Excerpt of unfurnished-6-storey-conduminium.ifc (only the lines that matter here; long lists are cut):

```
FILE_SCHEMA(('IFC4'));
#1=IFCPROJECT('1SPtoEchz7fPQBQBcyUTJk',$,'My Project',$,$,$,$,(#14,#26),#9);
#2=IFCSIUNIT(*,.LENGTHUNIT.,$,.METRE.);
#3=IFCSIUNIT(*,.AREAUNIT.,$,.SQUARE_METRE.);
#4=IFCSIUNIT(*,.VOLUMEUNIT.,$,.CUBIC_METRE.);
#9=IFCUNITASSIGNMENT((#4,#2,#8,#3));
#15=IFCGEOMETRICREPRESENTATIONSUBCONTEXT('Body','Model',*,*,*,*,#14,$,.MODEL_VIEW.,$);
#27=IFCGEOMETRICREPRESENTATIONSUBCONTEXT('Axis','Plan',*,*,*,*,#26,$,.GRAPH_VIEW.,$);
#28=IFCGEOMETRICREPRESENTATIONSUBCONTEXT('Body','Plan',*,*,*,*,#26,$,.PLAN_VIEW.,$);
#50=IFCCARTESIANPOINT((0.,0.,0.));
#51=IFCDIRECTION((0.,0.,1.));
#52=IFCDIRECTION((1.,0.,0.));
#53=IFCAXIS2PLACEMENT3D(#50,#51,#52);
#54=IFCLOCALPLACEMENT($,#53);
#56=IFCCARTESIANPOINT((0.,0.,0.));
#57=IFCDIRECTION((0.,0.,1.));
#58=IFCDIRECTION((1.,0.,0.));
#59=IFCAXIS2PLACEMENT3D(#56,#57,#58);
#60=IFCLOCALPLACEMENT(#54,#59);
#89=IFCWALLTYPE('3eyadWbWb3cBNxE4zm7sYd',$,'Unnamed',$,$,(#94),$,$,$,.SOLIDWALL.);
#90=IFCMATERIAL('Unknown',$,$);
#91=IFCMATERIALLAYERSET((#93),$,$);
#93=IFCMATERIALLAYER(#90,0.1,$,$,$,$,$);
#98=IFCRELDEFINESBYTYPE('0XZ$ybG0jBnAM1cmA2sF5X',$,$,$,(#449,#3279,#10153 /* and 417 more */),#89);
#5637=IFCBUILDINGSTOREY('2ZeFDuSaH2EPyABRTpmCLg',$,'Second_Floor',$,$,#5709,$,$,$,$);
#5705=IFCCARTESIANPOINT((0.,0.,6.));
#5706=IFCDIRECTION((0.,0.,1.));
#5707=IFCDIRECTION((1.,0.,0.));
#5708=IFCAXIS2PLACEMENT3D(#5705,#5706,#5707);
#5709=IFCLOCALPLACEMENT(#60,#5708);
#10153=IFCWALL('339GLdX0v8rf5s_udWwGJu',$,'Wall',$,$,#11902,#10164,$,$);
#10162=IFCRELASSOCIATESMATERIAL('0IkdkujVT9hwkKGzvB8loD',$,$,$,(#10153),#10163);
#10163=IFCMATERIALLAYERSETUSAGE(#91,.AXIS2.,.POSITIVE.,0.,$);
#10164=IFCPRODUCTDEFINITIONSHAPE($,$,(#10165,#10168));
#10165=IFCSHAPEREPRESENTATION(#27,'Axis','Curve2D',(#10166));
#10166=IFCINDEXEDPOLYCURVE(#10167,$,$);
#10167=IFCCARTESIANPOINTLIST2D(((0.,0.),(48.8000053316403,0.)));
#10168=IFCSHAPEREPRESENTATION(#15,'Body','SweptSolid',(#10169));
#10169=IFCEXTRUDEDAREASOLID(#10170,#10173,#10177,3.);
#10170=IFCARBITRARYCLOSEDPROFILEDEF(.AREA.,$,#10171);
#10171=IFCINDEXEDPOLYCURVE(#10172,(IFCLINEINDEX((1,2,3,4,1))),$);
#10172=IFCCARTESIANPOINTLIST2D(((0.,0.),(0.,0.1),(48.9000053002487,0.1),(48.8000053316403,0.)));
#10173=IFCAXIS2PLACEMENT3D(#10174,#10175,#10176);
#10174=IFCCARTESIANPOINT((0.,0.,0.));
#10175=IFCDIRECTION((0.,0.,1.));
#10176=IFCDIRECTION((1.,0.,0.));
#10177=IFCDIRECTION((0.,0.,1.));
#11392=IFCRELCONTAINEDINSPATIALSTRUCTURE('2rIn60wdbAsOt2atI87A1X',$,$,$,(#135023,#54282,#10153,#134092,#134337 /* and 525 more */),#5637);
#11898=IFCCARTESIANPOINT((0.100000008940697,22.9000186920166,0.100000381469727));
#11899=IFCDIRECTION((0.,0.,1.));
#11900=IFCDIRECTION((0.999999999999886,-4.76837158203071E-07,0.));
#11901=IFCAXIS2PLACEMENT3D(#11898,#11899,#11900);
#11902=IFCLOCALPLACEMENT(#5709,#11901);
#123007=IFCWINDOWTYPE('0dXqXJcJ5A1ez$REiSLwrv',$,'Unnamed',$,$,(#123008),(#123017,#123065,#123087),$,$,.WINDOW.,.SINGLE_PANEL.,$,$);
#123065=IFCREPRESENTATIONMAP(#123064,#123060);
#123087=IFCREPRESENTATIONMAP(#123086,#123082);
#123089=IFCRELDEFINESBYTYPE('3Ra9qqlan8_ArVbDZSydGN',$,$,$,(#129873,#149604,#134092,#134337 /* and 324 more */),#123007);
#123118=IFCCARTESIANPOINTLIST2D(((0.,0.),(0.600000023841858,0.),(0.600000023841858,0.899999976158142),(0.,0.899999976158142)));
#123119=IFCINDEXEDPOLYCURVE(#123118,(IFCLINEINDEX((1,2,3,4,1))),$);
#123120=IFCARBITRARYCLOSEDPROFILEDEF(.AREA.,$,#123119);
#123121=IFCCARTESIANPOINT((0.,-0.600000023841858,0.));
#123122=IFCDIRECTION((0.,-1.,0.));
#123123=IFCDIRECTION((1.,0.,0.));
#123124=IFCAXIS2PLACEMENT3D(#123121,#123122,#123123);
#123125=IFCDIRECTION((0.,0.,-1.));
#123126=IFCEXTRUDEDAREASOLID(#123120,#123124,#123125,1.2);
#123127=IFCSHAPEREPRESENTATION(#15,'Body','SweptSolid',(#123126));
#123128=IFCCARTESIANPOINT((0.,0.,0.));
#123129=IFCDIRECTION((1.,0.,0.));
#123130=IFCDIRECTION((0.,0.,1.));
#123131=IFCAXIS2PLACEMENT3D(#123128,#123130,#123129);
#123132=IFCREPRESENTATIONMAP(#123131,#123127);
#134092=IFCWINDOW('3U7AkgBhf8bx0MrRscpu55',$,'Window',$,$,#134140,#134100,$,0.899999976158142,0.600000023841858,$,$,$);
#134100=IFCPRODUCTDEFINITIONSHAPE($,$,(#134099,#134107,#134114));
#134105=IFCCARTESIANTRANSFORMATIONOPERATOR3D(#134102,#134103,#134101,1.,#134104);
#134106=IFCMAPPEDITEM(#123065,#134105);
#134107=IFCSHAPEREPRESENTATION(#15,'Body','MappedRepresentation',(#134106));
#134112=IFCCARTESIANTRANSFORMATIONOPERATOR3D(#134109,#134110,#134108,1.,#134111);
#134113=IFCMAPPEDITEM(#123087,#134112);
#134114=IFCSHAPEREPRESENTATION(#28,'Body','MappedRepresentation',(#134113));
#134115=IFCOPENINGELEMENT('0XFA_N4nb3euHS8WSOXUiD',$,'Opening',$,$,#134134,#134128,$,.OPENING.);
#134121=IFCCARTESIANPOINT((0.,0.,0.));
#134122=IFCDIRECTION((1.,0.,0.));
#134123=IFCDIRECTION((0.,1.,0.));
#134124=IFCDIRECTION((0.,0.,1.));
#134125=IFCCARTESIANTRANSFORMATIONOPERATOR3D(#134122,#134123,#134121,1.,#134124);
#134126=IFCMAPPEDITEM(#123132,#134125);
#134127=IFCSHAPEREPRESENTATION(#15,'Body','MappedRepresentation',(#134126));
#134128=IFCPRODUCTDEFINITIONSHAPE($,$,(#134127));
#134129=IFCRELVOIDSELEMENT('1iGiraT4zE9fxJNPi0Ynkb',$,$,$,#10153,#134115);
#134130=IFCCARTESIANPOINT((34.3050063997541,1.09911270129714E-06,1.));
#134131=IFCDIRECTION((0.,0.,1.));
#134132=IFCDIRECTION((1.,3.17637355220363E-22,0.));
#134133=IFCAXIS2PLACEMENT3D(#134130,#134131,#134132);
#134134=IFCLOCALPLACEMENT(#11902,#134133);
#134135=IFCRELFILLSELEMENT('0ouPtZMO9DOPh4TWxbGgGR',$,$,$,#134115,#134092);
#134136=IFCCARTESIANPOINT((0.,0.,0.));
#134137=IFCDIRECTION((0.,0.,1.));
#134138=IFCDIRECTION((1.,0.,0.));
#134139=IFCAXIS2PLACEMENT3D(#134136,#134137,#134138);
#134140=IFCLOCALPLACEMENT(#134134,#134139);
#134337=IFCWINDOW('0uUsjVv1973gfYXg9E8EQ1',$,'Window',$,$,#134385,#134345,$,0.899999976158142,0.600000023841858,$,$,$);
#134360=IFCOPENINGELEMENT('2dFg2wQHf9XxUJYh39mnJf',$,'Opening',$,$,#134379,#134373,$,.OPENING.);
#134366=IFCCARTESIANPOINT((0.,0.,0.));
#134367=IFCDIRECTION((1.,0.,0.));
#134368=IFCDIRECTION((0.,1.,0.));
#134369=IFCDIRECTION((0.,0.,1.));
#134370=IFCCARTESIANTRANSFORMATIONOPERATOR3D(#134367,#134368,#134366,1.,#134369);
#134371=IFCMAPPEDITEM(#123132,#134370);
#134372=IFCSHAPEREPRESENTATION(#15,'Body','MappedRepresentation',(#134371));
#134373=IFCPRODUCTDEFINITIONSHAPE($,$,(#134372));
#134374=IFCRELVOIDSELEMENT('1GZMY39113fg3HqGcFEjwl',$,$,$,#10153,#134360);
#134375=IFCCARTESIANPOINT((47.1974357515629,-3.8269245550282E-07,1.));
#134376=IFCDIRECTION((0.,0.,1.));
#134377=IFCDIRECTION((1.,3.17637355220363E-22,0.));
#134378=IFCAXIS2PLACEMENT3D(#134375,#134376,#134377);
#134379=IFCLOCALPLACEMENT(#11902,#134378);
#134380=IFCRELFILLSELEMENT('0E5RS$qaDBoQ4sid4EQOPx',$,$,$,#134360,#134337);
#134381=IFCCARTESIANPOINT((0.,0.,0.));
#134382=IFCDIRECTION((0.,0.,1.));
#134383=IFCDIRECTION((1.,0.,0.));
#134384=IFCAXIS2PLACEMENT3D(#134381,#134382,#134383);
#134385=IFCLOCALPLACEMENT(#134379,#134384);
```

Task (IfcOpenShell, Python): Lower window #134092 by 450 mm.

```python
import numpy as np
import ifcopenshell
import ifcopenshell.api.geometry
import ifcopenshell.util.placement
import ifcopenshell.util.unit

model = ifcopenshell.open("unfurnished-6-storey-conduminium.ifc")
unit_scale = ifcopenshell.util.unit.calculate_unit_scale(model)

window = model.by_id(134092)
opening = window.FillsVoids[0].RelatingOpeningElement
dz = -0.45 / unit_scale

shift = np.array([0.0, 0.0, dz])
# The window is placed relative to its opening, so it follows when the opening moves.
matrix = ifcopenshell.util.placement.get_local_placement(opening.ObjectPlacement)
matrix[:3, 3] += shift
ifcopenshell.api.geometry.edit_object_placement(
    model, product=opening, matrix=matrix, is_si=False, should_transform_children=True
)

print(f"moved by {dz * unit_scale:+.3f} m")

model.write("unfurnished-6-storey-conduminium_rev.ifc")
```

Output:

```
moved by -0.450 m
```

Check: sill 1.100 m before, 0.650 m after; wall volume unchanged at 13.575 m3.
